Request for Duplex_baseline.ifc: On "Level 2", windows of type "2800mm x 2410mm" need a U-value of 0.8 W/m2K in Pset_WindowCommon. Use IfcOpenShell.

First a look at what the model holds.

```python
import ifcopenshell
import ifcopenshell.util.element

model = ifcopenshell.open("Duplex_baseline.ifc")
print(model.schema)
storey = next(s for s in model.by_type("IfcBuildingStorey") if s.Name == "Level 2")
windows = [e for e in ifcopenshell.util.element.get_decomposition(storey) if e.is_a("IfcWindow")]
seen = {}
for e in windows:
    element_type = ifcopenshell.util.element.get_type(e)
    key = (element_type.Name if element_type != e and element_type else None, ifcopenshell.util.element.get_pset(e, "Pset_WindowCommon", "ThermalTransmittance"))
    seen[key] = seen.get(key, 0) + 1
for (name, value), count in sorted(seen.items(), key=str):
    print(count, "x", name, "|", value)
```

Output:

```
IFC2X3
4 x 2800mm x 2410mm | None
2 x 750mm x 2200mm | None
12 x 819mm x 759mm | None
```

```python
import ifcopenshell
import ifcopenshell.api.pset
import ifcopenshell.util.element

model = ifcopenshell.open("Duplex_baseline.ifc")

storey = next(s for s in model.by_type("IfcBuildingStorey") if s.Name == "Level 2")
windows = [e for e in ifcopenshell.util.element.get_decomposition(storey) if e.is_a("IfcWindow")]

count = 0
for e in windows:
    element_type = ifcopenshell.util.element.get_type(e)
    if element_type in (None, e) or element_type.Name != "2800mm x 2410mm":
        continue
    # add_pset returns the element's existing set when there is one.
    pset = ifcopenshell.api.pset.add_pset(model, product=e, name="Pset_WindowCommon")
    ifcopenshell.api.pset.edit_pset(model, pset=pset, properties={"ThermalTransmittance": 0.8})
    count += 1

print(count, "windows updated")

model.write("Duplex_baseline-out.ifc")
```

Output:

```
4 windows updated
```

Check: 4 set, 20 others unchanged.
